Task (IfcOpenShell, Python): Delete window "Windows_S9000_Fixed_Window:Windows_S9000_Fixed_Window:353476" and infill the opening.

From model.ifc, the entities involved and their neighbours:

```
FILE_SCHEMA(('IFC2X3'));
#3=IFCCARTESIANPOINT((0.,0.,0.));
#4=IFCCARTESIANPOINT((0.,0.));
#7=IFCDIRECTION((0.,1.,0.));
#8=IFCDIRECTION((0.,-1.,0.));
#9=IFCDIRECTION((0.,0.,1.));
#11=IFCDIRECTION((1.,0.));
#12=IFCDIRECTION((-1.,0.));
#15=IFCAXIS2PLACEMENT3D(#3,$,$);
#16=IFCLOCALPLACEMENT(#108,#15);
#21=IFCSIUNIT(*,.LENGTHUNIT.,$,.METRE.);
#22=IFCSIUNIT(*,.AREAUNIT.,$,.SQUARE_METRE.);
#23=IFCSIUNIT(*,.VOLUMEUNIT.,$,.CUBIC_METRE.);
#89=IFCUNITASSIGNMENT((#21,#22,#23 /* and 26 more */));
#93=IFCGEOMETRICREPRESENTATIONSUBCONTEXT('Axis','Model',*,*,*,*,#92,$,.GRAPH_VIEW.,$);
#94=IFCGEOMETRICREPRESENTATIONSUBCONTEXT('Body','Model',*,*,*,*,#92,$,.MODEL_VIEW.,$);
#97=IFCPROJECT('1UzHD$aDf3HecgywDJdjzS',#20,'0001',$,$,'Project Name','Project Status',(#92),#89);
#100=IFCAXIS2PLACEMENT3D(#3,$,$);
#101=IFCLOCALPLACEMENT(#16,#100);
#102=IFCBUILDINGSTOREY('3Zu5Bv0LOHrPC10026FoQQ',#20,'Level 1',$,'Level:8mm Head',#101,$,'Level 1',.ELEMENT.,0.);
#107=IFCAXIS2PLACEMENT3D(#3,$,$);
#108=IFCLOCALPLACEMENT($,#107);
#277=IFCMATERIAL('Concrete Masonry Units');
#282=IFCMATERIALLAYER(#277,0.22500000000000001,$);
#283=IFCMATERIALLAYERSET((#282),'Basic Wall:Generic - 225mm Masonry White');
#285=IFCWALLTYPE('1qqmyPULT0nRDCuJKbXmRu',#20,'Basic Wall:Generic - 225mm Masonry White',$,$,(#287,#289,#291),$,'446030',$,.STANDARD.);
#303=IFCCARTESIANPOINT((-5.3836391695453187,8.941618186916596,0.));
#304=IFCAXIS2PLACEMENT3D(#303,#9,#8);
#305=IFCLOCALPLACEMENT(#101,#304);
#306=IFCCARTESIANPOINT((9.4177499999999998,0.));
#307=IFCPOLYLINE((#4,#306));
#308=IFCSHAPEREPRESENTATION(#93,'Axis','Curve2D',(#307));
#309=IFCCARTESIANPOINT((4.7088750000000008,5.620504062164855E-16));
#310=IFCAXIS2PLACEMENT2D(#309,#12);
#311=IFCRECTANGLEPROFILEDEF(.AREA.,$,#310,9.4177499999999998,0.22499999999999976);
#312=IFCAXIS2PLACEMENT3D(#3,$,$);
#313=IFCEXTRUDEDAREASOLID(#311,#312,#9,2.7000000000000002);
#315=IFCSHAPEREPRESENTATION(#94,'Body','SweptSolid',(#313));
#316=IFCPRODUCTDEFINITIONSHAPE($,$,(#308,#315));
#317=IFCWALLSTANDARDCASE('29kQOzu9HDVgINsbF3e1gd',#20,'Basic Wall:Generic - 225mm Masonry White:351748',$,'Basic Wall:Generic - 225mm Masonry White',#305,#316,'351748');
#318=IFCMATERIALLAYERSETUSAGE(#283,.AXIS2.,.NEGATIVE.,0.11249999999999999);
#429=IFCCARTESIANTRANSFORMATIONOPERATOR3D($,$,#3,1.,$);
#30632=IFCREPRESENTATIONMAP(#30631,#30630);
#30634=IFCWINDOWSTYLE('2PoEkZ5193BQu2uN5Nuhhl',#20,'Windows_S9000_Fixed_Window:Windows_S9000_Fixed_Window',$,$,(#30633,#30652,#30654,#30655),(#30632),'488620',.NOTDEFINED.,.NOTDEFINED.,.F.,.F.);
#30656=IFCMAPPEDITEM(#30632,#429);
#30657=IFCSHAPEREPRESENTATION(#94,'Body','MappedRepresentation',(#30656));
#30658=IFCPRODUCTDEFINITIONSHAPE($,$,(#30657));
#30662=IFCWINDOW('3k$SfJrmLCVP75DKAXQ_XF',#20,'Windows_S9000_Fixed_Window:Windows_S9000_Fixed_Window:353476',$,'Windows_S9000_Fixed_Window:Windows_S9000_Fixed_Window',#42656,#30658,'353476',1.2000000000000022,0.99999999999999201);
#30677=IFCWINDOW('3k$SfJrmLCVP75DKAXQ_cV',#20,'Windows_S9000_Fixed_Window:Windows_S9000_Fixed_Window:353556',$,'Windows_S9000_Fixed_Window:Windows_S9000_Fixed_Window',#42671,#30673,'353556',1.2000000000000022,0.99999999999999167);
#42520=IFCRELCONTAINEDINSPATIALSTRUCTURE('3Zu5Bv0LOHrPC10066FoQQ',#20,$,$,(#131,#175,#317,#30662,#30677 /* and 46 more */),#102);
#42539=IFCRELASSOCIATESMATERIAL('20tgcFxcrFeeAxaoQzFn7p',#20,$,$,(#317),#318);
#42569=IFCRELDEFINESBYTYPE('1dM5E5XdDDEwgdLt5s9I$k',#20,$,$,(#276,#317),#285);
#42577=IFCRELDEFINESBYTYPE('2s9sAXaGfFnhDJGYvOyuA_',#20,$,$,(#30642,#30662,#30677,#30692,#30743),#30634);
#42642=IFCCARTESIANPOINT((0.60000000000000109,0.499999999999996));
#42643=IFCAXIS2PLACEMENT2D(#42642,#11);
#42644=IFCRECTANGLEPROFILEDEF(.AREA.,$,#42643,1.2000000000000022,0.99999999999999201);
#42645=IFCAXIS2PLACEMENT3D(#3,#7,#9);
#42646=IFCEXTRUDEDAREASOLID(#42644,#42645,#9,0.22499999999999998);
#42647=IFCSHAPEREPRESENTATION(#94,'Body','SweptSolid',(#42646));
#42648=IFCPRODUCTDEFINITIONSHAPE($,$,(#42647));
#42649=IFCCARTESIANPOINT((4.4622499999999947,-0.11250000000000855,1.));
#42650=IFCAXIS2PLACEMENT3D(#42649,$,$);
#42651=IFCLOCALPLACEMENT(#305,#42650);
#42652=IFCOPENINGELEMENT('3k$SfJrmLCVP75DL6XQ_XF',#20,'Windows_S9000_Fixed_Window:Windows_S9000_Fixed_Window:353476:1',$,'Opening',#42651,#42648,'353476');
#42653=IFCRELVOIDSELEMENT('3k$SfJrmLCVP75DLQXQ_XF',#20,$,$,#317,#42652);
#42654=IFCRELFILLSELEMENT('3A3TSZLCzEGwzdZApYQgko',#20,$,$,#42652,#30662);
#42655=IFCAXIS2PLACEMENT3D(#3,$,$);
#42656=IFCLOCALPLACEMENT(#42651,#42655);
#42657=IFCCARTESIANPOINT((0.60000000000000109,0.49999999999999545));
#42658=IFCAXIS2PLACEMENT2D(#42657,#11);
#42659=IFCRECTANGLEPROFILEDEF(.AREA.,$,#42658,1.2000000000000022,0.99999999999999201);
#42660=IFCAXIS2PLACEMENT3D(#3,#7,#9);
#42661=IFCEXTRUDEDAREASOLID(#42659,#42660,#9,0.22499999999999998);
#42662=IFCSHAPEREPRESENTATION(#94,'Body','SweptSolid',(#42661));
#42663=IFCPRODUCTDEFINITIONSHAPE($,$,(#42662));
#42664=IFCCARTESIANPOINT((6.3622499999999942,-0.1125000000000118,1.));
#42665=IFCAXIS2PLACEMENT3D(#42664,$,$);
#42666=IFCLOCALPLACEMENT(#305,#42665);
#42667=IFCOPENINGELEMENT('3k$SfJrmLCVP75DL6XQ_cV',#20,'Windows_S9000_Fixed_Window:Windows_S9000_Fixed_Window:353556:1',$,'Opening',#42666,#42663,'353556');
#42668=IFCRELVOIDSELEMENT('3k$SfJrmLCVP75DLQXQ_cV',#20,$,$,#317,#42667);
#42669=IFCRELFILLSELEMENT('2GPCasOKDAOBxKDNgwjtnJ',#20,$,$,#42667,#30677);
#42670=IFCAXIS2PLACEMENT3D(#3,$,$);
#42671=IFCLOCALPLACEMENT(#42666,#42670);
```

```python
import ifcopenshell
import ifcopenshell.api.feature
import ifcopenshell.api.root
import ifcopenshell.geom
import ifcopenshell.util.shape

model = ifcopenshell.open("model.ifc")
settings = ifcopenshell.geom.settings()


def volume(element):
    """Net volume in cubic metres, openings subtracted."""
    shape = ifcopenshell.geom.create_shape(settings, element)
    return ifcopenshell.util.shape.get_volume(shape.geometry)


window = model.by_guid("3k$SfJrmLCVP75DKAXQ_XF")
opening = window.FillsVoids[0].RelatingOpeningElement
wall = opening.VoidsElements[0].RelatingBuildingElement
before = volume(wall)

ifcopenshell.api.root.remove_product(model, product=window)
ifcopenshell.api.feature.remove_feature(model, feature=opening)

after = volume(wall)

print(f"wall volume {before:.3f} -> {after:.3f} m3")

model.write("model_rev.ifc")
```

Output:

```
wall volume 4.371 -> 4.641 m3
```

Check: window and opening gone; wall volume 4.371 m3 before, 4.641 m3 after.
